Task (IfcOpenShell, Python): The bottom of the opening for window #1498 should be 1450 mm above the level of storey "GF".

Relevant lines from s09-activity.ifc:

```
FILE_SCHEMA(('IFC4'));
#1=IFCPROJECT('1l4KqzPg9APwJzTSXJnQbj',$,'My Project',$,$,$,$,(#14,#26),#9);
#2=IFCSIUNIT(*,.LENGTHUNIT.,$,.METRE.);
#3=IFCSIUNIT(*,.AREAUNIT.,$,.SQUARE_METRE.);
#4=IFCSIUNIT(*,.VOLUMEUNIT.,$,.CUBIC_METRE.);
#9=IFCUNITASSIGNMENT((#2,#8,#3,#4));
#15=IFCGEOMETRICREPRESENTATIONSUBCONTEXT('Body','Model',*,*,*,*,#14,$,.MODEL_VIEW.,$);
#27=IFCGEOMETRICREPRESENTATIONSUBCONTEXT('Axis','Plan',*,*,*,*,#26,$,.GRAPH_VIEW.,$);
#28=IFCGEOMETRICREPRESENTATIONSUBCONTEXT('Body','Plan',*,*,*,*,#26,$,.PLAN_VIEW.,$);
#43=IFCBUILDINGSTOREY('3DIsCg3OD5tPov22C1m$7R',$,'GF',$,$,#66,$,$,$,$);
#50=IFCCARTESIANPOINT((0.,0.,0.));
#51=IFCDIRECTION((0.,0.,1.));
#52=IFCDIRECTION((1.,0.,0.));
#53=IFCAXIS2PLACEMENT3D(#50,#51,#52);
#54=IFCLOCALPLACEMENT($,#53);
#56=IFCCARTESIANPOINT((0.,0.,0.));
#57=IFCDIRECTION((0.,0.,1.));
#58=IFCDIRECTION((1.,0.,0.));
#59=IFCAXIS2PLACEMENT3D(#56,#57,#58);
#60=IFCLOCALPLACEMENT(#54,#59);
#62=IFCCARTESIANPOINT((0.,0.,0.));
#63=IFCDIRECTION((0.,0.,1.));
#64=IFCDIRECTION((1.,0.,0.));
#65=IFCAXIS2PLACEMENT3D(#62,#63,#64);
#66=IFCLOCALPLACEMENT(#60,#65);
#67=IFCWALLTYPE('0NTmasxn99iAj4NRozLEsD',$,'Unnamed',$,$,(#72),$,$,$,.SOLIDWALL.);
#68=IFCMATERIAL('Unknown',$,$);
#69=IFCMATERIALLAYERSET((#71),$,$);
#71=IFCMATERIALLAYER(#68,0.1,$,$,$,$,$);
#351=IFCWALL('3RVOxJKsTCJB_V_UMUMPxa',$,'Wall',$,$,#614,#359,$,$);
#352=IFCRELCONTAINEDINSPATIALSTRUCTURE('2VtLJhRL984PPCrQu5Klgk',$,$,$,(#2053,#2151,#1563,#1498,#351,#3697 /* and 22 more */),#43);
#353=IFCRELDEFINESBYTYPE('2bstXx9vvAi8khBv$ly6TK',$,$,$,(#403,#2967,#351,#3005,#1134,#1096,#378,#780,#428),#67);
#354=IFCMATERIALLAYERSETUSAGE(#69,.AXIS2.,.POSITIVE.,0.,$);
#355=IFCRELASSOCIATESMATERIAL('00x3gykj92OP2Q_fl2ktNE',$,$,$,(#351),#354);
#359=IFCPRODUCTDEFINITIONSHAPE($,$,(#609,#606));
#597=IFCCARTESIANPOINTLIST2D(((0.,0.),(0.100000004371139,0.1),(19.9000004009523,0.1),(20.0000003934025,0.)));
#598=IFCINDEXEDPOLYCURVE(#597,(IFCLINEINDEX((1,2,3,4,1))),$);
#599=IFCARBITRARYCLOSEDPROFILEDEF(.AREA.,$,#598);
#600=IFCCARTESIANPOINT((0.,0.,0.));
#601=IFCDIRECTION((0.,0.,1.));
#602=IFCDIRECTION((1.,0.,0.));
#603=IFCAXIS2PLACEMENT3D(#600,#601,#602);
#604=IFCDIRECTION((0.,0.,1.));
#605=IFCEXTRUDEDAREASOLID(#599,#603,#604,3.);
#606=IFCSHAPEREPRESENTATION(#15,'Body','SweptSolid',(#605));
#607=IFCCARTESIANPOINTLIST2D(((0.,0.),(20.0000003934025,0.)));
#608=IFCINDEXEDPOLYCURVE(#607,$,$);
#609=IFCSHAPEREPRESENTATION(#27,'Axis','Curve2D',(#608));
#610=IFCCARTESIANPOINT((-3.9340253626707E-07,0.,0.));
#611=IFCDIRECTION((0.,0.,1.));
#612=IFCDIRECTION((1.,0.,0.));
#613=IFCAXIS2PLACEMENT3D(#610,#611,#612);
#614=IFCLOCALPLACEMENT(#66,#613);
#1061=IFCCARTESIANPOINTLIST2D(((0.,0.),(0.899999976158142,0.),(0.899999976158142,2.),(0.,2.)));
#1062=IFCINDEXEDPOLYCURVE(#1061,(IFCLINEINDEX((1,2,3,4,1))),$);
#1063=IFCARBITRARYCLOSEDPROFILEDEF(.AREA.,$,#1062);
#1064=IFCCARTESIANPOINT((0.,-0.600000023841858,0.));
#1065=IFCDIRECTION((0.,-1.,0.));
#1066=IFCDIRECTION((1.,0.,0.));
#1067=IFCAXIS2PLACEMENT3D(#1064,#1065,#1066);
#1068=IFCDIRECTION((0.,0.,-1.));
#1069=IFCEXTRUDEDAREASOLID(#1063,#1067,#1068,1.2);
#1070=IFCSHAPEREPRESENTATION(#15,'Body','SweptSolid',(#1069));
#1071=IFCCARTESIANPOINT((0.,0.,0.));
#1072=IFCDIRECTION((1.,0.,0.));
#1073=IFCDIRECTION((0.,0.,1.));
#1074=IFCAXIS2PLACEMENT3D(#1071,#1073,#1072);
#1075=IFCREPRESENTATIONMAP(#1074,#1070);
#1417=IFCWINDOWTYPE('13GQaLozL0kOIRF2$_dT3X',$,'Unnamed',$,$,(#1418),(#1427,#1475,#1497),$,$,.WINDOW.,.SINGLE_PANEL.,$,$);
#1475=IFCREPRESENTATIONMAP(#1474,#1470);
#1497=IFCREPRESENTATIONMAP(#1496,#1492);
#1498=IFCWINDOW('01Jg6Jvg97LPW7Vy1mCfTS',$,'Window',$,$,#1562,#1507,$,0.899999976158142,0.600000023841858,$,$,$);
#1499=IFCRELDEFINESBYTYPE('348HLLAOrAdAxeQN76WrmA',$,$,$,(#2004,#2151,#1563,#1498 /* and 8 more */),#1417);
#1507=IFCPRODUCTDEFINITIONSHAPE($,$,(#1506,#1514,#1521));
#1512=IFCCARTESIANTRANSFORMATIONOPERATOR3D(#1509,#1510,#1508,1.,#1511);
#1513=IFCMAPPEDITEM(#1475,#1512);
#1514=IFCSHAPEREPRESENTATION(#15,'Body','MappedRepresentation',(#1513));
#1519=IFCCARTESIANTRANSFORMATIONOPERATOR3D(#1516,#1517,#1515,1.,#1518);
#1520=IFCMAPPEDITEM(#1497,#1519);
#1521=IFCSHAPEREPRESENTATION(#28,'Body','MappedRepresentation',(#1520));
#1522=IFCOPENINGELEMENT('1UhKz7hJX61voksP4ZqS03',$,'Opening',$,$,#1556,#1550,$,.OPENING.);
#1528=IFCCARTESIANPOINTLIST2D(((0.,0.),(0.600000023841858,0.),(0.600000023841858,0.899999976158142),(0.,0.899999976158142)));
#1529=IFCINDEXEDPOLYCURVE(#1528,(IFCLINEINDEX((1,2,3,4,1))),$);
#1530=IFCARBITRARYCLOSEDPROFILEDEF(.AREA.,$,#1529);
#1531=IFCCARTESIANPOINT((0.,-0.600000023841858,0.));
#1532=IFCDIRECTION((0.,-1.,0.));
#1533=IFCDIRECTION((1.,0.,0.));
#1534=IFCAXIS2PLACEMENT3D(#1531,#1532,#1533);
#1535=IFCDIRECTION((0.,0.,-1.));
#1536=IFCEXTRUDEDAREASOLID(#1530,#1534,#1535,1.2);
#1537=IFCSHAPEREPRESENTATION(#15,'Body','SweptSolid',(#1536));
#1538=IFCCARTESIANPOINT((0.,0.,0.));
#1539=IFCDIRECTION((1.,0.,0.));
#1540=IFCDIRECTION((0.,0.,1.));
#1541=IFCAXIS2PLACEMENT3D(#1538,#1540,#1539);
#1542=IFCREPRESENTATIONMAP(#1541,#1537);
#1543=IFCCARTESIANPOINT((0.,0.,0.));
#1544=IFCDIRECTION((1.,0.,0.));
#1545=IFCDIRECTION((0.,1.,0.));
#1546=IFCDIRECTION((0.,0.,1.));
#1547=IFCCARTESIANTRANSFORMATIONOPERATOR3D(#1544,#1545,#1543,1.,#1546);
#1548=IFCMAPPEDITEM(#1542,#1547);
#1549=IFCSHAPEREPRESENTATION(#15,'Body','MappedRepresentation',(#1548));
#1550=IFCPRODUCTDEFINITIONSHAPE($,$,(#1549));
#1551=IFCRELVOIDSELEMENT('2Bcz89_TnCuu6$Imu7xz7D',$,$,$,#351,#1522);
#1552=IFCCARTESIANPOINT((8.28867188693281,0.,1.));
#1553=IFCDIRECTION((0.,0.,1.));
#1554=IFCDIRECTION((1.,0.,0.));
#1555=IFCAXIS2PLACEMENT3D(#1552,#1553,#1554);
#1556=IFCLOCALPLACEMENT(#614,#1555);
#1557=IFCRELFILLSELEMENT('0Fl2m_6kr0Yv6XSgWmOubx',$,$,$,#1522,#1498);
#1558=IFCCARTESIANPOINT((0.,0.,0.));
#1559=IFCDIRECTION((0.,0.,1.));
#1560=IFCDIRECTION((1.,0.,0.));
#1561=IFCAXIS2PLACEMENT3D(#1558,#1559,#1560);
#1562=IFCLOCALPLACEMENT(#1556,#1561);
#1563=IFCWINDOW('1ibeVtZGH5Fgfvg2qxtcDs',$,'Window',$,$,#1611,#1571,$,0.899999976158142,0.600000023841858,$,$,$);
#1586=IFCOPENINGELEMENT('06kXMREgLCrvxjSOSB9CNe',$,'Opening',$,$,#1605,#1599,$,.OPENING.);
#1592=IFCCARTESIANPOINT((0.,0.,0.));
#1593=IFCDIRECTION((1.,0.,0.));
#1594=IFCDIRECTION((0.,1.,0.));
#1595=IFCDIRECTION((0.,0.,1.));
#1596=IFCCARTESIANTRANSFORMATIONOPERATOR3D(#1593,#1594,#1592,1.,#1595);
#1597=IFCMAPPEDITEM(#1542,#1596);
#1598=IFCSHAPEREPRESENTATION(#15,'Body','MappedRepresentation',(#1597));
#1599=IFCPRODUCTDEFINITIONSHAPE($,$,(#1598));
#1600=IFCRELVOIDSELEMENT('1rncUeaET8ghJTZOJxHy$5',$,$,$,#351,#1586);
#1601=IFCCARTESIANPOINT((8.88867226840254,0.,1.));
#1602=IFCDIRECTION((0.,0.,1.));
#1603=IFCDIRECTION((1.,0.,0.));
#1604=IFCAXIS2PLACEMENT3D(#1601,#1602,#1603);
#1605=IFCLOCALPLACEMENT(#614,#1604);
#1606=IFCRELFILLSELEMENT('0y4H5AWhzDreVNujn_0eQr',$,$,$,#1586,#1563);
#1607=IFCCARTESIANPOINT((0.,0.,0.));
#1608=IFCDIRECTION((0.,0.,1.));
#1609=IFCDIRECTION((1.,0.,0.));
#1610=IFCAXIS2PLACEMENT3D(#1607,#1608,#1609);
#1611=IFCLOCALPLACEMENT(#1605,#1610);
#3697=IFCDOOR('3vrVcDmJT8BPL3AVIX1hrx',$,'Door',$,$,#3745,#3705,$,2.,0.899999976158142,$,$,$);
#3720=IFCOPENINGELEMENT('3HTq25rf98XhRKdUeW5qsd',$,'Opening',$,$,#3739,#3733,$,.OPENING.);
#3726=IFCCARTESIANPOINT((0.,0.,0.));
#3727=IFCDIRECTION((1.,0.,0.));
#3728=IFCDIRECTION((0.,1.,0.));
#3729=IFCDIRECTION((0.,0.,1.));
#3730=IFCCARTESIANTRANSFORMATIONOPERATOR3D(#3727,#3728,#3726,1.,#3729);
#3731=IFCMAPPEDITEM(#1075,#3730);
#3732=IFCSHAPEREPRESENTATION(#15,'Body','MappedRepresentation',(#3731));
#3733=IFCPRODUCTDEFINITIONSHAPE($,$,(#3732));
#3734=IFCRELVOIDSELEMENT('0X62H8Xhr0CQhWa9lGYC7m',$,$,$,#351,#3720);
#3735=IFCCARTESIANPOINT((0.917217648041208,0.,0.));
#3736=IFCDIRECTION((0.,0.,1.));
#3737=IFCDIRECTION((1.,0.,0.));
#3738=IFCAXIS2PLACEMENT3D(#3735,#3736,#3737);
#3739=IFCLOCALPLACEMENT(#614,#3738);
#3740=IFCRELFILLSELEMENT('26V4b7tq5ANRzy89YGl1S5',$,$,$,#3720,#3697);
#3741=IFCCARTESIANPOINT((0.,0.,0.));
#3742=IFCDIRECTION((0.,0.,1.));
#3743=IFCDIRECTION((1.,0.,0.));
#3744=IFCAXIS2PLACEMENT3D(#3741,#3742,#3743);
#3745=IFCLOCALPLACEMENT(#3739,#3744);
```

```python
import numpy as np
import ifcopenshell
import ifcopenshell.api.geometry
import ifcopenshell.geom
import ifcopenshell.util.element
import ifcopenshell.util.placement
import ifcopenshell.util.shape
import ifcopenshell.util.unit

model = ifcopenshell.open("s09-activity.ifc")
unit_scale = ifcopenshell.util.unit.calculate_unit_scale(model)

window = model.by_id(1498)
opening = window.FillsVoids[0].RelatingOpeningElement
storey = ifcopenshell.util.element.get_container(window, ifc_class="IfcBuildingStorey")
level = ifcopenshell.util.placement.get_local_placement(storey.ObjectPlacement)[2, 3]

# The opening's origin need not be at the sill, so measure its lowest point.
shape = ifcopenshell.geom.create_shape(ifcopenshell.geom.settings(), opening)
bottom = ifcopenshell.util.shape.get_shape_bottom_elevation(shape, shape.geometry) / unit_scale
dz = level + 1.45 - bottom

shift = np.array([0.0, 0.0, dz])
# The window is placed relative to its opening, so it follows when the opening moves.
matrix = ifcopenshell.util.placement.get_local_placement(opening.ObjectPlacement)
matrix[:3, 3] += shift
ifcopenshell.api.geometry.edit_object_placement(
    model, product=opening, matrix=matrix, is_si=False, should_transform_children=True
)

print(f"moved by {dz * unit_scale:+.3f} m")

model.write("s09-activity_edited.ifc")
```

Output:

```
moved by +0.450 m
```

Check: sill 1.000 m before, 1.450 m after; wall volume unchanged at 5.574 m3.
